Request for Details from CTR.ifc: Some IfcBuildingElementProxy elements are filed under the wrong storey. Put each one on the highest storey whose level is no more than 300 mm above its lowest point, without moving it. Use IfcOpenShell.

First a look at what the model holds.

```python
import ifcopenshell
import ifcopenshell.util.element
import ifcopenshell.util.placement

model = ifcopenshell.open("Details from CTR.ifc")
print(model.schema)
for storey in model.by_type("IfcBuildingStorey"):
    level = ifcopenshell.util.placement.get_storey_elevation(storey)
    count = sum(e.is_a("IfcBuildingElementProxy") for e in ifcopenshell.util.element.get_contained(storey))
    print(storey.id(), storey.Name, round(level, 3), count, sep=" | ")
```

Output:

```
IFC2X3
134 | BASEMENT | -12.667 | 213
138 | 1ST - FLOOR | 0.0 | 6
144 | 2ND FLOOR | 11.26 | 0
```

```python
import ifcopenshell
import ifcopenshell.api.spatial
import ifcopenshell.geom
import ifcopenshell.util.element
import ifcopenshell.util.placement
import ifcopenshell.util.shape
import ifcopenshell.util.unit

model = ifcopenshell.open("Details from CTR.ifc")
unit_scale = ifcopenshell.util.unit.calculate_unit_scale(model)
settings = ifcopenshell.geom.settings()

levels = sorted(
    ((ifcopenshell.util.placement.get_storey_elevation(s) * unit_scale, s) for s in model.by_type("IfcBuildingStorey")),
    key=lambda pair: pair[0],
)

for e in model.by_type("IfcBuildingElementProxy"):
    current = e.ContainedInStructure[0].RelatingStructure if e.ContainedInStructure else None
    if current is None or not current.is_a("IfcBuildingStorey"):
        continue
    shape = ifcopenshell.geom.create_shape(settings, e)
    bottom = ifcopenshell.util.shape.get_shape_bottom_elevation(shape, shape.geometry)
    below = [s for level, s in levels if level <= bottom + 0.3]
    storey = below[-1] if below else levels[0][1]
    if storey != current:
        # assign_container keeps the world position.
        ifcopenshell.api.spatial.assign_container(model, products=[e], relating_structure=storey)
        print(e.id(), current.Name, "->", storey.Name)

model.write("Details from CTR_edited.ifc")
```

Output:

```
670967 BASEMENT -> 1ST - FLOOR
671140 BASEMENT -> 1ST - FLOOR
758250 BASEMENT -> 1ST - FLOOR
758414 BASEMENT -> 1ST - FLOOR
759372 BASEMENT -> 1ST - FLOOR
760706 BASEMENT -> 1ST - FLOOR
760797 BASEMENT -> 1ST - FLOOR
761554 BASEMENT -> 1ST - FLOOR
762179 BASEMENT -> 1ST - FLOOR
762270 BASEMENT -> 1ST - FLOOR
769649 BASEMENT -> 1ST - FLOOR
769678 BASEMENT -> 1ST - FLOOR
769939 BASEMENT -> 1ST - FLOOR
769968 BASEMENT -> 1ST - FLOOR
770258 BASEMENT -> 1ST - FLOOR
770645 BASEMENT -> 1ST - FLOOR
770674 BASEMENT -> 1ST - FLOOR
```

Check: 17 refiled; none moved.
